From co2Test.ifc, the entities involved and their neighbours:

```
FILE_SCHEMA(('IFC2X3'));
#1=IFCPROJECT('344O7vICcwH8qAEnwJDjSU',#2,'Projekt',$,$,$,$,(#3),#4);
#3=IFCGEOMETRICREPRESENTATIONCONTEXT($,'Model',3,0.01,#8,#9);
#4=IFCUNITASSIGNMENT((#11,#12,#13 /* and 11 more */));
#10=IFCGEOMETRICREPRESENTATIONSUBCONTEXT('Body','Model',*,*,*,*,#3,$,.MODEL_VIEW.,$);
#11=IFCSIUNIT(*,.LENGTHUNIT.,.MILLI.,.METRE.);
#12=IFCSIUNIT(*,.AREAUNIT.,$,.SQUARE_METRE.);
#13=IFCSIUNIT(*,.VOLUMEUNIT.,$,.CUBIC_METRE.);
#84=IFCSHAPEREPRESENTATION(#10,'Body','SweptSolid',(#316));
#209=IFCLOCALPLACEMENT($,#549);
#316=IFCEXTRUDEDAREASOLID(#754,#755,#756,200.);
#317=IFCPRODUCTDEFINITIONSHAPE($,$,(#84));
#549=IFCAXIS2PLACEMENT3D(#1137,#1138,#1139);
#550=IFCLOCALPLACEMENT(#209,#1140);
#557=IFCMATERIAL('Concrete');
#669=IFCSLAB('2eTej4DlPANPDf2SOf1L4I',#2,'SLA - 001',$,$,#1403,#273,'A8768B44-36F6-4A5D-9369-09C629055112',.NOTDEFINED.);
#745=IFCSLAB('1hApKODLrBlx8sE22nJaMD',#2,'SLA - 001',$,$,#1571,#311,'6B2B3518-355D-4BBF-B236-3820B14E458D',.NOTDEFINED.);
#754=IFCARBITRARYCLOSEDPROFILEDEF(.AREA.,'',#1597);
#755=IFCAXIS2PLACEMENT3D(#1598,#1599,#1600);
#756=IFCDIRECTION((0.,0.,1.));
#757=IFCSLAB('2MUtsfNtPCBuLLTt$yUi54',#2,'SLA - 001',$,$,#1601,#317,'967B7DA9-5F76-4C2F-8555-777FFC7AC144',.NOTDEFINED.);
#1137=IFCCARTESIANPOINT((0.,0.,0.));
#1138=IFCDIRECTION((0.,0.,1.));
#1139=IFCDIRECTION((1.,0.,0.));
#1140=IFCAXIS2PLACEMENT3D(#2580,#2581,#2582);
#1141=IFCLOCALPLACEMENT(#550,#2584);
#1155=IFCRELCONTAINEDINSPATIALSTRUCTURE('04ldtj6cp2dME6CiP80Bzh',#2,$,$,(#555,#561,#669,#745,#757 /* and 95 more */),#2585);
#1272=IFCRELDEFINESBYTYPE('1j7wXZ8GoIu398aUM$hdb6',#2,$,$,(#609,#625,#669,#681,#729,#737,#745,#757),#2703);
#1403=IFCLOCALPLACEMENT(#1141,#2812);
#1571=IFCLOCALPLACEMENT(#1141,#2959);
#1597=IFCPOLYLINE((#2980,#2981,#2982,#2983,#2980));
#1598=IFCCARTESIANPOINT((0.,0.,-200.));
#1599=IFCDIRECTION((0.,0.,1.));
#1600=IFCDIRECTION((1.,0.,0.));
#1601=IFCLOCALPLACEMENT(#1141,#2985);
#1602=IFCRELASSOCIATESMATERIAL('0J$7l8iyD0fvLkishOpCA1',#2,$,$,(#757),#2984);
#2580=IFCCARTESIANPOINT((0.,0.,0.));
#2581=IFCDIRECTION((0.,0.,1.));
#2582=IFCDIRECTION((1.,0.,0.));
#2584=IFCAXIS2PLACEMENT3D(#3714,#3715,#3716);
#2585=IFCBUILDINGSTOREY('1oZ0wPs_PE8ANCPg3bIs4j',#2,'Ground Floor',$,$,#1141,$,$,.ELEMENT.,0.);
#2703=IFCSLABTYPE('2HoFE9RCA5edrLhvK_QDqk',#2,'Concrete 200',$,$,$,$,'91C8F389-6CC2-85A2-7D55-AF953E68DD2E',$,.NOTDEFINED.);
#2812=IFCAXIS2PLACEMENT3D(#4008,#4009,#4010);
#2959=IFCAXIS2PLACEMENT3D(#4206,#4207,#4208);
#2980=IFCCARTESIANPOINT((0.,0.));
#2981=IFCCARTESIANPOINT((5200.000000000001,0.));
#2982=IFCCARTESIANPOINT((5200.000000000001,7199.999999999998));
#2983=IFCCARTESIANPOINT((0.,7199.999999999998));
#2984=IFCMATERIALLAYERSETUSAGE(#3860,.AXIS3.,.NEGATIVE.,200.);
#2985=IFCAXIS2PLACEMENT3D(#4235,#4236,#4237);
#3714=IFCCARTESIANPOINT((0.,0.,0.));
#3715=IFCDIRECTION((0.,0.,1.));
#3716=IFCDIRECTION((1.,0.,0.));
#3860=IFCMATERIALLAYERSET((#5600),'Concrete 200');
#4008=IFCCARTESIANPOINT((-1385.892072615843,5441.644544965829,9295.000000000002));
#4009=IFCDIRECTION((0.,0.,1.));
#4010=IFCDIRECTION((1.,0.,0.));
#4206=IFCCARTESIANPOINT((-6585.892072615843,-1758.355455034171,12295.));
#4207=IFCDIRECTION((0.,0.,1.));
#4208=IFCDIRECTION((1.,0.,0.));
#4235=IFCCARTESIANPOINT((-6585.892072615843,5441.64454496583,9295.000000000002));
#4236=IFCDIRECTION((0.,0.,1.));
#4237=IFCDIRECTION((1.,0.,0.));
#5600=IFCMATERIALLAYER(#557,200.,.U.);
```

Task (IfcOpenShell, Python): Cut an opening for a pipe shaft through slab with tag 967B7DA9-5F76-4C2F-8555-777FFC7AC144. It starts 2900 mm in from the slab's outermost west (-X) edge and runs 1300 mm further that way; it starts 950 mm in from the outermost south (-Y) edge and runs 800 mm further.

```python
import numpy as np
import ifcopenshell
import ifcopenshell.api.feature
import ifcopenshell.api.geometry
import ifcopenshell.api.root
import ifcopenshell.geom
import ifcopenshell.util.placement
import ifcopenshell.util.representation
import ifcopenshell.util.shape
import ifcopenshell.util.unit

model = ifcopenshell.open("co2Test.ifc")
unit_scale = ifcopenshell.util.unit.calculate_unit_scale(model)
settings = ifcopenshell.geom.settings()


def volume(element):
    """Net volume in cubic metres, openings subtracted."""
    shape = ifcopenshell.geom.create_shape(settings, element)
    return ifcopenshell.util.shape.get_volume(shape.geometry)


slab = model.by_guid("2MUtsfNtPCBuLLTt$yUi54")
before = volume(slab)

# Extent in the slab's own axes, in metres. The edges named are its -X and -Y sides.
slab_shape = ifcopenshell.geom.create_shape(settings, slab)
vertices = ifcopenshell.util.shape.get_vertices(slab_shape.geometry)
x_min, y_min, bottom = vertices.min(axis=0)
top = vertices[:, 2].max()

opening = ifcopenshell.api.root.create_entity(model, ifc_class="IfcOpeningElement", name="Pipe shaft opening")
context = ifcopenshell.util.representation.get_context(model, "Model", "Body", "MODEL_VIEW")
width, depth = 1.3, 0.8
outline = [(0.0, 0.0), (width, 0.0), (width, depth), (0.0, depth), (0.0, 0.0)]
# Overshoot both faces by 50 mm so the cut is clean.
shape = ifcopenshell.api.geometry.add_slab_representation(
    model, context=context, depth=top - bottom + 0.1, polyline=outline
)
ifcopenshell.api.geometry.assign_representation(model, product=opening, representation=shape)

matrix = ifcopenshell.util.placement.get_local_placement(slab.ObjectPlacement)
matrix[:, 3] = matrix @ np.append(np.array([x_min + 2.9, y_min + 0.95, bottom - 0.05]) / unit_scale, 1.0)
ifcopenshell.api.geometry.edit_object_placement(model, product=opening, matrix=matrix, is_si=False)
ifcopenshell.api.feature.add_feature(model, feature=opening, element=slab)

after = volume(slab)

print(f"slab volume {before:.3f} -> {after:.3f} m3")

model.write("co2Test_updated.ifc")
```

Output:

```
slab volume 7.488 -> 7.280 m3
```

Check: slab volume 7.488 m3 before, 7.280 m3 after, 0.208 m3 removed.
